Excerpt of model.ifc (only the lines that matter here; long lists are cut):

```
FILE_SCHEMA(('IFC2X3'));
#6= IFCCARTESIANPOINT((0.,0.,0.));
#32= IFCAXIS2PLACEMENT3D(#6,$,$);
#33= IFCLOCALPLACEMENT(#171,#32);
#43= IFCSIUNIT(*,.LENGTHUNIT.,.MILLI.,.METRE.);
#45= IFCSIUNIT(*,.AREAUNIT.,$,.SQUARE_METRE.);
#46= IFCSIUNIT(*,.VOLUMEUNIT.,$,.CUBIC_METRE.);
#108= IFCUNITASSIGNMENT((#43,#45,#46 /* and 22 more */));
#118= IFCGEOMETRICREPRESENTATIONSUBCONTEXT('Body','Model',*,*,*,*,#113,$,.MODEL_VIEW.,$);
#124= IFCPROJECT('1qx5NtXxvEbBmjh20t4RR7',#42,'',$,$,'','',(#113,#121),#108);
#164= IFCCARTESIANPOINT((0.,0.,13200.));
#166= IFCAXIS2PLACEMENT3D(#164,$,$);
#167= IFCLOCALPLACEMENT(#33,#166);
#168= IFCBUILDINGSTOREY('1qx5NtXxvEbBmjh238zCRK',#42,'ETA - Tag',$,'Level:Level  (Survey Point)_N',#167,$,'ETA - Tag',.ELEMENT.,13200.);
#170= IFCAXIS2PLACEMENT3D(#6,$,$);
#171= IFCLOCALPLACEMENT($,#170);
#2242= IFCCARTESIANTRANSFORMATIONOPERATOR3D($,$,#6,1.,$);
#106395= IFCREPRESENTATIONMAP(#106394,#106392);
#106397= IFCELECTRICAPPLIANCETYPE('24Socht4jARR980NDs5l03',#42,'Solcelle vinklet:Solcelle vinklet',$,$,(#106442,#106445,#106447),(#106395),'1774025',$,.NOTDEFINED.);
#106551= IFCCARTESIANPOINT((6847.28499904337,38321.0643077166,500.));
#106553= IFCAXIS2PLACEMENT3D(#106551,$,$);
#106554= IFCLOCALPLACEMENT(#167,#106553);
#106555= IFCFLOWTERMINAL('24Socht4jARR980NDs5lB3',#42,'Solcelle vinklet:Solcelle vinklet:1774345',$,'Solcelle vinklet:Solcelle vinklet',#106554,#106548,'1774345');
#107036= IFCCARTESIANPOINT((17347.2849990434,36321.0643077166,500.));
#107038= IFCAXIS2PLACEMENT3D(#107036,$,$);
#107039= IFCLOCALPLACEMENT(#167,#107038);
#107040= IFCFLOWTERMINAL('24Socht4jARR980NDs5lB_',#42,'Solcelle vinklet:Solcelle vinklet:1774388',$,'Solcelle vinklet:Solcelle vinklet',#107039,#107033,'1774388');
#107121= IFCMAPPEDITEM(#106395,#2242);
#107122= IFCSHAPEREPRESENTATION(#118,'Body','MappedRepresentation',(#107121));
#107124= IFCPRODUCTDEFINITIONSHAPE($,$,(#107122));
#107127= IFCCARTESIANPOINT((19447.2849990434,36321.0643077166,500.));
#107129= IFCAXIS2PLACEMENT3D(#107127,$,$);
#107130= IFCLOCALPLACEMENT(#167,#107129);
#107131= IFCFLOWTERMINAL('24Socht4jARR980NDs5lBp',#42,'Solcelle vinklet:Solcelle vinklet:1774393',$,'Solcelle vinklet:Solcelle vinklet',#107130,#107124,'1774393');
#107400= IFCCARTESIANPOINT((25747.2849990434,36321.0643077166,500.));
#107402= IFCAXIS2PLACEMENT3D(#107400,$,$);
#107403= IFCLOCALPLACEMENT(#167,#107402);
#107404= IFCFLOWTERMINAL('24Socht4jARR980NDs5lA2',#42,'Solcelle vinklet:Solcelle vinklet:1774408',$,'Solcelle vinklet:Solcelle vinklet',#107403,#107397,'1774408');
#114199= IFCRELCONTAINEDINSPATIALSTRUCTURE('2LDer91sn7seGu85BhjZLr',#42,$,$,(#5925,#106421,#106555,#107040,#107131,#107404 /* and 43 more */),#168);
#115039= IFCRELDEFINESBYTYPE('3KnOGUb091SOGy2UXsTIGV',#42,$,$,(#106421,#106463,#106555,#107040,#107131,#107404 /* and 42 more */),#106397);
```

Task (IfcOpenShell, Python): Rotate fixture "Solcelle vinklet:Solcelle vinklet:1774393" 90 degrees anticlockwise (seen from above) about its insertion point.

```python
import ifcopenshell
import ifcopenshell.api.geometry
import ifcopenshell.util.placement

model = ifcopenshell.open("model.ifc")

item = model.by_id(107131)
matrix = ifcopenshell.util.placement.get_local_placement(item.ObjectPlacement)
matrix = matrix @ ifcopenshell.util.placement.rotation(90, "Z")
ifcopenshell.api.geometry.edit_object_placement(model, product=item, matrix=matrix, is_si=False)

print(ifcopenshell.util.placement.get_local_placement(item.ObjectPlacement).round(3) + 0.0)

model.write("model_edited.ifc")
```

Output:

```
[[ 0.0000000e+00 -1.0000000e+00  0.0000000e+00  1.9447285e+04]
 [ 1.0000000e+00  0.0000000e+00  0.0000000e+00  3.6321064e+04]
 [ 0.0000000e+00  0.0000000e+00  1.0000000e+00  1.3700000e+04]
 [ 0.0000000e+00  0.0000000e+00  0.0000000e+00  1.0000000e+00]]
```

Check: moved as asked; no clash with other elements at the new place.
